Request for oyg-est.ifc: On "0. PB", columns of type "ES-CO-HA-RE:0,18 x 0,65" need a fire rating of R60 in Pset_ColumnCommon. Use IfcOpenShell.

First a look at what the model holds.

```python
import ifcopenshell
import ifcopenshell.util.element

model = ifcopenshell.open("oyg-est.ifc")
print(model.schema)
storey = next(s for s in model.by_type("IfcBuildingStorey") if s.Name == "0. PB")
columns = [e for e in ifcopenshell.util.element.get_decomposition(storey) if e.is_a("IfcColumn")]
seen = {}
for e in columns:
    element_type = ifcopenshell.util.element.get_type(e)
    key = (element_type.Name if element_type != e and element_type else None, ifcopenshell.util.element.get_pset(e, "Pset_ColumnCommon", "FireRating"))
    seen[key] = seen.get(key, 0) + 1
for (name, value), count in sorted(seen.items(), key=str):
    print(count, "x", name, "|", value)
```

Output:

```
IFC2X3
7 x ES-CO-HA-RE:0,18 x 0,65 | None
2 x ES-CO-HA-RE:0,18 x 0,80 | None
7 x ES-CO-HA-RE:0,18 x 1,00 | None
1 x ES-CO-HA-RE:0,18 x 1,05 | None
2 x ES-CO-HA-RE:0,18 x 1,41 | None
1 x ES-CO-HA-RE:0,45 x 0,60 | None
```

```python
import ifcopenshell
import ifcopenshell.api.pset
import ifcopenshell.util.element

model = ifcopenshell.open("oyg-est.ifc")

storey = next(s for s in model.by_type("IfcBuildingStorey") if s.Name == "0. PB")
columns = [e for e in ifcopenshell.util.element.get_decomposition(storey) if e.is_a("IfcColumn")]

count = 0
for e in columns:
    element_type = ifcopenshell.util.element.get_type(e)
    if element_type in (None, e) or element_type.Name != "ES-CO-HA-RE:0,18 x 0,65":
        continue
    # add_pset returns the element's existing set when there is one.
    pset = ifcopenshell.api.pset.add_pset(model, product=e, name="Pset_ColumnCommon")
    ifcopenshell.api.pset.edit_pset(model, pset=pset, properties={"FireRating": "R60"})
    count += 1

print(count, "columns updated")

model.write("oyg-est_rev.ifc")
```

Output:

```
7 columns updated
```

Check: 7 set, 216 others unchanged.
